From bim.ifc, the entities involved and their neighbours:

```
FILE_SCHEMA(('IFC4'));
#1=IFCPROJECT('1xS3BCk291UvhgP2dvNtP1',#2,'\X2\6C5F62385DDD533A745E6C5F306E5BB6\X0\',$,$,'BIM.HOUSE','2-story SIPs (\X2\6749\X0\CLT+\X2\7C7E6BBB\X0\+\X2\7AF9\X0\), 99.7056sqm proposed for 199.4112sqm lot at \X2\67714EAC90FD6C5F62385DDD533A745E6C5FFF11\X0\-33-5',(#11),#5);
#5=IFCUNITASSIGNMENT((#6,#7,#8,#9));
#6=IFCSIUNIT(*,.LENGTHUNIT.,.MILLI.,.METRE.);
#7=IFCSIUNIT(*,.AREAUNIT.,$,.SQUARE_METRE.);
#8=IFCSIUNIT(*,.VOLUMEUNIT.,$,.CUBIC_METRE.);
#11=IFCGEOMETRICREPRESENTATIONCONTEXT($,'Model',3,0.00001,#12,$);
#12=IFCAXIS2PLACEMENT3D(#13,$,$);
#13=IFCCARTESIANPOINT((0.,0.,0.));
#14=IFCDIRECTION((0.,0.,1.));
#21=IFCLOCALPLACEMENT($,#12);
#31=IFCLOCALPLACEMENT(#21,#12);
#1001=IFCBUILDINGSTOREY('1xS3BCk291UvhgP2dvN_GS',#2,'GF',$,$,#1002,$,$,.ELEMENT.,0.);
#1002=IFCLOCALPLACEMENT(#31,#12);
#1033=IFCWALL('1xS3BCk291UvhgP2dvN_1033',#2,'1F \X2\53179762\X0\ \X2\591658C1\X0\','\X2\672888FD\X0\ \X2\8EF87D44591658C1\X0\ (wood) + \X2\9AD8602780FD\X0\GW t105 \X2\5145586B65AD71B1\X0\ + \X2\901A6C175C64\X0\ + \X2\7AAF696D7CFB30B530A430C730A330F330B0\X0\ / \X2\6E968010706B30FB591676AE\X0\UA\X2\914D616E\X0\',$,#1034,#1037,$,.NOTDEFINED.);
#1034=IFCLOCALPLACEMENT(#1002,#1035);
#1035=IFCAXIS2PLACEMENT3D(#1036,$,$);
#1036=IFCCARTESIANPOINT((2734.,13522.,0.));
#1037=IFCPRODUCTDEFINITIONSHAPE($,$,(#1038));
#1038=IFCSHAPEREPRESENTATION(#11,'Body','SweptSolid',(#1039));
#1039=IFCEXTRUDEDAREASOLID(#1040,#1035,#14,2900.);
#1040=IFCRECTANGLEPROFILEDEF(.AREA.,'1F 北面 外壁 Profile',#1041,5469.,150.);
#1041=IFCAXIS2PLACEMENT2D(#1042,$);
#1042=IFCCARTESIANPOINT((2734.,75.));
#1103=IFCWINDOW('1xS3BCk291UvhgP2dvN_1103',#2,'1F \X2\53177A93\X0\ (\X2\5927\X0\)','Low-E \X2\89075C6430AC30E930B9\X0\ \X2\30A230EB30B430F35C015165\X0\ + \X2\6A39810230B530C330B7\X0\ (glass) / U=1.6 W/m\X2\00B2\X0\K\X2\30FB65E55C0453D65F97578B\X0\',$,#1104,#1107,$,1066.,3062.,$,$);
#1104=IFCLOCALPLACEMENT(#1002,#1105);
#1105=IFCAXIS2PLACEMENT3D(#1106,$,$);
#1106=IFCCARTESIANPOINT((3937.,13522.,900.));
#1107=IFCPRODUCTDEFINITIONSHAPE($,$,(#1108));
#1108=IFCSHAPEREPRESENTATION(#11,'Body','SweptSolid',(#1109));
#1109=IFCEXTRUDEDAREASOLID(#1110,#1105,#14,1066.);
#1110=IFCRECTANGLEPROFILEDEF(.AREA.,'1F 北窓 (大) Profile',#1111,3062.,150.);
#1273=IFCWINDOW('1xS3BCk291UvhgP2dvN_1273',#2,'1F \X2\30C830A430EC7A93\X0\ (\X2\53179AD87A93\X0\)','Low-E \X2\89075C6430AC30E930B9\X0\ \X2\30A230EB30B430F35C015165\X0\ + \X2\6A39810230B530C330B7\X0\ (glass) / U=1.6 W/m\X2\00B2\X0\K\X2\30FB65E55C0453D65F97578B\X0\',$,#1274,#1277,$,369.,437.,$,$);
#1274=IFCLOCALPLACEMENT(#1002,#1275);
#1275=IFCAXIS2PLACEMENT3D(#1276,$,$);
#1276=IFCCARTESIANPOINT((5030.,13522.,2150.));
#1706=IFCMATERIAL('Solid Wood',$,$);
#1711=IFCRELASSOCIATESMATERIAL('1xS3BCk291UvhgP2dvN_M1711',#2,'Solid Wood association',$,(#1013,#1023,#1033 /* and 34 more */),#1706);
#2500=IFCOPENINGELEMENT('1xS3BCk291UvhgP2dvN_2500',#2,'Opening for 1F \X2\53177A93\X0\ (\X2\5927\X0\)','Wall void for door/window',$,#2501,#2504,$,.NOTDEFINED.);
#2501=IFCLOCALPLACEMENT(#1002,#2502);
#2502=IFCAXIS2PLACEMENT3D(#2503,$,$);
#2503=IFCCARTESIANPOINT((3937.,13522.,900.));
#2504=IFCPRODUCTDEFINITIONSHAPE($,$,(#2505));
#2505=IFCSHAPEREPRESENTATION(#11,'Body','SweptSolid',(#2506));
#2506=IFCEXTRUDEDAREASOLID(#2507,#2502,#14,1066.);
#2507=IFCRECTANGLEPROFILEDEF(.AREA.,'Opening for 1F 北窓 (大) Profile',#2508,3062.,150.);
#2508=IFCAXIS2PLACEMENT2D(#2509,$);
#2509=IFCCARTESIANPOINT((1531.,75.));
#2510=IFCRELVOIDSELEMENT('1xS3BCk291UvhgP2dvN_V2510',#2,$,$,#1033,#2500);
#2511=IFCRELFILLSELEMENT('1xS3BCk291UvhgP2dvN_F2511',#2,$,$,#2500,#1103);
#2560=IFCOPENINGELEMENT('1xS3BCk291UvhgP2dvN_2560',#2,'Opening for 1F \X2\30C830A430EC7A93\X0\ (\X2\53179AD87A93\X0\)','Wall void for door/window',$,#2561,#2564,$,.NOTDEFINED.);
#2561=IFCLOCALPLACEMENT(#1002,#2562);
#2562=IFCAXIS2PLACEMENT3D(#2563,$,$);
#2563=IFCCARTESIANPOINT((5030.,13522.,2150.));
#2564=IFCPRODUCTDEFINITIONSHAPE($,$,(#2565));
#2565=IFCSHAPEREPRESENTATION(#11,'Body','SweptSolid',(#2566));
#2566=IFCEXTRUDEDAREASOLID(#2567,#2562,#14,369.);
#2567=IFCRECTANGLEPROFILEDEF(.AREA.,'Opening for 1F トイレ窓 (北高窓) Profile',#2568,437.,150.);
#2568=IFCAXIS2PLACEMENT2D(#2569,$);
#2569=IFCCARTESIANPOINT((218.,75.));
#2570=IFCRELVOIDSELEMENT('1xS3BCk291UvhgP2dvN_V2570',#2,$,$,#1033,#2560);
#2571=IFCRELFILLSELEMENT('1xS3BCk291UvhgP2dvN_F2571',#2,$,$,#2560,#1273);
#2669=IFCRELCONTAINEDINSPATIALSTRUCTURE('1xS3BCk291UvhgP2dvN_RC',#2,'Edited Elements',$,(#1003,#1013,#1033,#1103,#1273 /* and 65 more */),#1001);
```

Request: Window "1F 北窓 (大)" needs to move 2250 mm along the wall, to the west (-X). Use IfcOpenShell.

```python
import ifcopenshell
import ifcopenshell.api.geometry
import ifcopenshell.util.placement
import ifcopenshell.util.unit

model = ifcopenshell.open("bim.ifc")
unit_scale = ifcopenshell.util.unit.calculate_unit_scale(model)

window = model.by_guid("1xS3BCk291UvhgP2dvN_1103")
opening = window.FillsVoids[0].RelatingOpeningElement
wall = opening.VoidsElements[0].RelatingBuildingElement

wall_matrix = ifcopenshell.util.placement.get_local_placement(wall.ObjectPlacement)
shift = wall_matrix[:3, 0] * -2.25 / unit_scale
before = ifcopenshell.util.placement.get_local_placement(window.ObjectPlacement)[:3, 3].copy()

# The window is not placed relative to its opening, so move both.
for product in (opening, window):
    matrix = ifcopenshell.util.placement.get_local_placement(product.ObjectPlacement)
    matrix[:3, 3] += shift
    ifcopenshell.api.geometry.edit_object_placement(model, product=product, matrix=matrix, is_si=False)

after = ifcopenshell.util.placement.get_local_placement(window.ObjectPlacement)[:3, 3]
print("window moved by", (after - before).round(3) + 0.0)

model.write("bim_updated.ifc")
```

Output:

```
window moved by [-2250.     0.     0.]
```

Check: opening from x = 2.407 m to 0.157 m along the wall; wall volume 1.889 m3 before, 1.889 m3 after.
